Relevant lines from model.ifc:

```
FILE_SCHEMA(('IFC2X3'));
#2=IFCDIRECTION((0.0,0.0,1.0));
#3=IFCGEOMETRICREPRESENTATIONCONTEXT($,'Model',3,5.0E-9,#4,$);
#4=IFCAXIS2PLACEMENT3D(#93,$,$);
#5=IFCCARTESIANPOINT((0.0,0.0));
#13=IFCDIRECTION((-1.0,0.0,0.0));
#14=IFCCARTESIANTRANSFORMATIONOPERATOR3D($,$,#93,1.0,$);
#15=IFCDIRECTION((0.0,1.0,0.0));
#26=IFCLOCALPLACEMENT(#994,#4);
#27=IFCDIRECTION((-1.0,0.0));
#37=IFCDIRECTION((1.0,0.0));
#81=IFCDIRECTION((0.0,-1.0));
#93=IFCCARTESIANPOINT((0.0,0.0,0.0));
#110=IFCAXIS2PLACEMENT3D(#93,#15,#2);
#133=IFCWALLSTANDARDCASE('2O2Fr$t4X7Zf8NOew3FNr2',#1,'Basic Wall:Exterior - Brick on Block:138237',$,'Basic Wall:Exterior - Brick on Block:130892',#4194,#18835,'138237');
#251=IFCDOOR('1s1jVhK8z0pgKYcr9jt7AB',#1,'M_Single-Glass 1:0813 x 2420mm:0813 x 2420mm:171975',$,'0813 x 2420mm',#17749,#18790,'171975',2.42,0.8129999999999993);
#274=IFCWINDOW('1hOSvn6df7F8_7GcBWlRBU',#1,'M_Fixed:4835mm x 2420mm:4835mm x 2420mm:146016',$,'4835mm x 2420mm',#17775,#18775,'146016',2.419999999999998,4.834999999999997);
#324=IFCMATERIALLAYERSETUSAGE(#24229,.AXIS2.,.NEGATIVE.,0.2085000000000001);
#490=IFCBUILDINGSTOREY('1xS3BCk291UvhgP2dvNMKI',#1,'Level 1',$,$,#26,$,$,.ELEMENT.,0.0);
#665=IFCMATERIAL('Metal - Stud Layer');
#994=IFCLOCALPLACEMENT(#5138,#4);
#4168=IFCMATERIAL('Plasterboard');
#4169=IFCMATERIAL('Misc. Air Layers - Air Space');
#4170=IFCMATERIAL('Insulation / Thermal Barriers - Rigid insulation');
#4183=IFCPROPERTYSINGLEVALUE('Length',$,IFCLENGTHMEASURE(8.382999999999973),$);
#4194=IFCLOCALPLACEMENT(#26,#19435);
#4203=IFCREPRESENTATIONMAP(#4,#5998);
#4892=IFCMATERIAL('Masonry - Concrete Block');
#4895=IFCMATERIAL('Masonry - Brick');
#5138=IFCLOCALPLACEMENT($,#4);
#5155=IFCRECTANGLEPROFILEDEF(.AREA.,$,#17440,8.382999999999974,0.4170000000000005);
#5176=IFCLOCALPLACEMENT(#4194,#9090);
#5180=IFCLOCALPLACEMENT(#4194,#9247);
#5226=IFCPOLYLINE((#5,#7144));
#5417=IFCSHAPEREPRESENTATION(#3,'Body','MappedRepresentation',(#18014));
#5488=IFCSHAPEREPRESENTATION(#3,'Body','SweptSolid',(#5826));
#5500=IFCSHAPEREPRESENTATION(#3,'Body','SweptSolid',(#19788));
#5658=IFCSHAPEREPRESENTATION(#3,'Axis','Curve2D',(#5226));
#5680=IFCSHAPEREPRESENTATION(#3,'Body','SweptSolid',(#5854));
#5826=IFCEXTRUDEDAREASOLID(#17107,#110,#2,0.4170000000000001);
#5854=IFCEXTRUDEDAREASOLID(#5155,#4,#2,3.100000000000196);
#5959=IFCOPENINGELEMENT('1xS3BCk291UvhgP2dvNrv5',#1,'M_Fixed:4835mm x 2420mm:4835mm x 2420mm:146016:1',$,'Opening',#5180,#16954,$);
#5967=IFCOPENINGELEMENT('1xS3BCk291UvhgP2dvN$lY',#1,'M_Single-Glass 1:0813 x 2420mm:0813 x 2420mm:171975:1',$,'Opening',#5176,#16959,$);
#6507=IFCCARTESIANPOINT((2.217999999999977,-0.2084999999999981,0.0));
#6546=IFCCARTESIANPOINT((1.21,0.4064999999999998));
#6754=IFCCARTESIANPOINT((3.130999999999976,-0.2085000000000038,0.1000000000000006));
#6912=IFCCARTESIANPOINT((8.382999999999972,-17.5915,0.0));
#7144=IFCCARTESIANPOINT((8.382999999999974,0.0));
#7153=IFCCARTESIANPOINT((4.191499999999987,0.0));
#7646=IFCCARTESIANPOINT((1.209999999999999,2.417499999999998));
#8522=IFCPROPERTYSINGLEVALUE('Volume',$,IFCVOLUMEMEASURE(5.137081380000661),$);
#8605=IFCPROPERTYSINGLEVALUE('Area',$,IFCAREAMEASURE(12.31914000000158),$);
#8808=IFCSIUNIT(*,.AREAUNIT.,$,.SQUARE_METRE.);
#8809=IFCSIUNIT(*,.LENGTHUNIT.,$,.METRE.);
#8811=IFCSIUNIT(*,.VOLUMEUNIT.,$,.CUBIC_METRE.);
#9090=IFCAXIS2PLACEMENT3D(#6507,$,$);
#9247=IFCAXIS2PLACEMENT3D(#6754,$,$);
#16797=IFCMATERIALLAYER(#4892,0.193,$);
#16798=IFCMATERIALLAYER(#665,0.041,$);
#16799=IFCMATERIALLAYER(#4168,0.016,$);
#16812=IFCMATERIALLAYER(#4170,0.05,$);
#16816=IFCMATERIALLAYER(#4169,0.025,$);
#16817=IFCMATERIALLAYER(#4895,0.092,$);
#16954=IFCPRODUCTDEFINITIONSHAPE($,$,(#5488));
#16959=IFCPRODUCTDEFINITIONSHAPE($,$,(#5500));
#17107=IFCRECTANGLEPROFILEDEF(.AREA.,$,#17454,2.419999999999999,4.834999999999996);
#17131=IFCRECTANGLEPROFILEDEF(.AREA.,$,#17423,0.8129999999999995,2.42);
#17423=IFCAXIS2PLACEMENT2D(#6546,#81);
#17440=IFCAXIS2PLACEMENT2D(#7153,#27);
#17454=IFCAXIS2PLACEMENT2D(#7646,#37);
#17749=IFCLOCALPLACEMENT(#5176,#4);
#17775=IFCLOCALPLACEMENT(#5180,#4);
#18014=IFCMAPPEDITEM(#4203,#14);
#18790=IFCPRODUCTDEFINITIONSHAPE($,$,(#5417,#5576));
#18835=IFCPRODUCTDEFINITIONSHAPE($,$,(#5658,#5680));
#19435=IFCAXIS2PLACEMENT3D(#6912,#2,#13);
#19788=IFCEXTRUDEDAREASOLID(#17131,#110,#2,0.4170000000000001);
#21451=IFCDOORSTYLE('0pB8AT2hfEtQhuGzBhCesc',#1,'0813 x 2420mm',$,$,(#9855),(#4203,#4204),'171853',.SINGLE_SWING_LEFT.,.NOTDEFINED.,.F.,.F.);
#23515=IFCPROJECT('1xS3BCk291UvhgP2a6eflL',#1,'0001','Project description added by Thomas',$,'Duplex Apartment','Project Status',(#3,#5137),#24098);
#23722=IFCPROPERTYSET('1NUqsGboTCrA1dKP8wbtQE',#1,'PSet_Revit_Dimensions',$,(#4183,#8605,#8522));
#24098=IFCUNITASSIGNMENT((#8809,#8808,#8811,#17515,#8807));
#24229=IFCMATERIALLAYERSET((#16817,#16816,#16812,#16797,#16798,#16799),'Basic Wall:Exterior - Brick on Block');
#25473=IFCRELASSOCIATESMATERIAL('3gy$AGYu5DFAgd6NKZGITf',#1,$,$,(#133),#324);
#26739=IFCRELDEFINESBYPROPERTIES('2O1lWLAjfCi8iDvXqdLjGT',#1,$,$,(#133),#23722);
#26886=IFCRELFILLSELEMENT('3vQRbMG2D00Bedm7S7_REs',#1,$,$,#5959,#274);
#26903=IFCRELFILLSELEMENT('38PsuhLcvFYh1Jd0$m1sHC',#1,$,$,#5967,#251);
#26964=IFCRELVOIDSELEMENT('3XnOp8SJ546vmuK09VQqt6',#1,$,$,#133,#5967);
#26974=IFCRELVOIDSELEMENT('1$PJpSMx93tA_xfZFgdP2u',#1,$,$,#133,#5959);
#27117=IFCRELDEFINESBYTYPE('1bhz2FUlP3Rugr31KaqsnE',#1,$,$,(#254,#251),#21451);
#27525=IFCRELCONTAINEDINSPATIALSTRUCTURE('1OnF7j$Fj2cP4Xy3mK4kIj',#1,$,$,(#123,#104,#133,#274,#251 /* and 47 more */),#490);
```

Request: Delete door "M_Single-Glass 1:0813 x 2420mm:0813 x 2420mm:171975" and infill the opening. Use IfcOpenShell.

```python
import ifcopenshell
import ifcopenshell.api.feature
import ifcopenshell.api.pset
import ifcopenshell.api.root
import ifcopenshell.geom
import ifcopenshell.util.element
import ifcopenshell.util.shape
import ifcopenshell.util.unit

model = ifcopenshell.open("model.ifc")
area_scale = ifcopenshell.util.unit.calculate_unit_scale(model, "AREAUNIT")
volume_scale = ifcopenshell.util.unit.calculate_unit_scale(model, "VOLUMEUNIT")
settings = ifcopenshell.geom.settings()


def volume(element):
    """Net volume in cubic metres, openings subtracted."""
    shape = ifcopenshell.geom.create_shape(settings, element)
    return ifcopenshell.util.shape.get_volume(shape.geometry)


door = model.by_id(251)
opening = door.FillsVoids[0].RelatingOpeningElement
wall = opening.VoidsElements[0].RelatingBuildingElement
before = volume(wall)

ifcopenshell.api.root.remove_product(model, product=door)
ifcopenshell.api.feature.remove_feature(model, feature=opening)

after = volume(wall)
thickness = 0.417  # wall thickness in metres

# Update the wall's stored quantities.
pset = model.by_id(ifcopenshell.util.element.get_pset(wall, "PSet_Revit_Dimensions", should_inherit=False)["id"])
ifcopenshell.api.pset.edit_pset(model, pset=pset, properties={
    "Area": model.create_entity("IfcAreaMeasure", after / thickness / area_scale),
    "Volume": model.create_entity("IfcVolumeMeasure", after / volume_scale),
})

print(f"wall volume {before:.3f} -> {after:.3f} m3")

model.write("model_v2.ifc")
```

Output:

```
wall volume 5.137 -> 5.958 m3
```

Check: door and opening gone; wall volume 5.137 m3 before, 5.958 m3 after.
